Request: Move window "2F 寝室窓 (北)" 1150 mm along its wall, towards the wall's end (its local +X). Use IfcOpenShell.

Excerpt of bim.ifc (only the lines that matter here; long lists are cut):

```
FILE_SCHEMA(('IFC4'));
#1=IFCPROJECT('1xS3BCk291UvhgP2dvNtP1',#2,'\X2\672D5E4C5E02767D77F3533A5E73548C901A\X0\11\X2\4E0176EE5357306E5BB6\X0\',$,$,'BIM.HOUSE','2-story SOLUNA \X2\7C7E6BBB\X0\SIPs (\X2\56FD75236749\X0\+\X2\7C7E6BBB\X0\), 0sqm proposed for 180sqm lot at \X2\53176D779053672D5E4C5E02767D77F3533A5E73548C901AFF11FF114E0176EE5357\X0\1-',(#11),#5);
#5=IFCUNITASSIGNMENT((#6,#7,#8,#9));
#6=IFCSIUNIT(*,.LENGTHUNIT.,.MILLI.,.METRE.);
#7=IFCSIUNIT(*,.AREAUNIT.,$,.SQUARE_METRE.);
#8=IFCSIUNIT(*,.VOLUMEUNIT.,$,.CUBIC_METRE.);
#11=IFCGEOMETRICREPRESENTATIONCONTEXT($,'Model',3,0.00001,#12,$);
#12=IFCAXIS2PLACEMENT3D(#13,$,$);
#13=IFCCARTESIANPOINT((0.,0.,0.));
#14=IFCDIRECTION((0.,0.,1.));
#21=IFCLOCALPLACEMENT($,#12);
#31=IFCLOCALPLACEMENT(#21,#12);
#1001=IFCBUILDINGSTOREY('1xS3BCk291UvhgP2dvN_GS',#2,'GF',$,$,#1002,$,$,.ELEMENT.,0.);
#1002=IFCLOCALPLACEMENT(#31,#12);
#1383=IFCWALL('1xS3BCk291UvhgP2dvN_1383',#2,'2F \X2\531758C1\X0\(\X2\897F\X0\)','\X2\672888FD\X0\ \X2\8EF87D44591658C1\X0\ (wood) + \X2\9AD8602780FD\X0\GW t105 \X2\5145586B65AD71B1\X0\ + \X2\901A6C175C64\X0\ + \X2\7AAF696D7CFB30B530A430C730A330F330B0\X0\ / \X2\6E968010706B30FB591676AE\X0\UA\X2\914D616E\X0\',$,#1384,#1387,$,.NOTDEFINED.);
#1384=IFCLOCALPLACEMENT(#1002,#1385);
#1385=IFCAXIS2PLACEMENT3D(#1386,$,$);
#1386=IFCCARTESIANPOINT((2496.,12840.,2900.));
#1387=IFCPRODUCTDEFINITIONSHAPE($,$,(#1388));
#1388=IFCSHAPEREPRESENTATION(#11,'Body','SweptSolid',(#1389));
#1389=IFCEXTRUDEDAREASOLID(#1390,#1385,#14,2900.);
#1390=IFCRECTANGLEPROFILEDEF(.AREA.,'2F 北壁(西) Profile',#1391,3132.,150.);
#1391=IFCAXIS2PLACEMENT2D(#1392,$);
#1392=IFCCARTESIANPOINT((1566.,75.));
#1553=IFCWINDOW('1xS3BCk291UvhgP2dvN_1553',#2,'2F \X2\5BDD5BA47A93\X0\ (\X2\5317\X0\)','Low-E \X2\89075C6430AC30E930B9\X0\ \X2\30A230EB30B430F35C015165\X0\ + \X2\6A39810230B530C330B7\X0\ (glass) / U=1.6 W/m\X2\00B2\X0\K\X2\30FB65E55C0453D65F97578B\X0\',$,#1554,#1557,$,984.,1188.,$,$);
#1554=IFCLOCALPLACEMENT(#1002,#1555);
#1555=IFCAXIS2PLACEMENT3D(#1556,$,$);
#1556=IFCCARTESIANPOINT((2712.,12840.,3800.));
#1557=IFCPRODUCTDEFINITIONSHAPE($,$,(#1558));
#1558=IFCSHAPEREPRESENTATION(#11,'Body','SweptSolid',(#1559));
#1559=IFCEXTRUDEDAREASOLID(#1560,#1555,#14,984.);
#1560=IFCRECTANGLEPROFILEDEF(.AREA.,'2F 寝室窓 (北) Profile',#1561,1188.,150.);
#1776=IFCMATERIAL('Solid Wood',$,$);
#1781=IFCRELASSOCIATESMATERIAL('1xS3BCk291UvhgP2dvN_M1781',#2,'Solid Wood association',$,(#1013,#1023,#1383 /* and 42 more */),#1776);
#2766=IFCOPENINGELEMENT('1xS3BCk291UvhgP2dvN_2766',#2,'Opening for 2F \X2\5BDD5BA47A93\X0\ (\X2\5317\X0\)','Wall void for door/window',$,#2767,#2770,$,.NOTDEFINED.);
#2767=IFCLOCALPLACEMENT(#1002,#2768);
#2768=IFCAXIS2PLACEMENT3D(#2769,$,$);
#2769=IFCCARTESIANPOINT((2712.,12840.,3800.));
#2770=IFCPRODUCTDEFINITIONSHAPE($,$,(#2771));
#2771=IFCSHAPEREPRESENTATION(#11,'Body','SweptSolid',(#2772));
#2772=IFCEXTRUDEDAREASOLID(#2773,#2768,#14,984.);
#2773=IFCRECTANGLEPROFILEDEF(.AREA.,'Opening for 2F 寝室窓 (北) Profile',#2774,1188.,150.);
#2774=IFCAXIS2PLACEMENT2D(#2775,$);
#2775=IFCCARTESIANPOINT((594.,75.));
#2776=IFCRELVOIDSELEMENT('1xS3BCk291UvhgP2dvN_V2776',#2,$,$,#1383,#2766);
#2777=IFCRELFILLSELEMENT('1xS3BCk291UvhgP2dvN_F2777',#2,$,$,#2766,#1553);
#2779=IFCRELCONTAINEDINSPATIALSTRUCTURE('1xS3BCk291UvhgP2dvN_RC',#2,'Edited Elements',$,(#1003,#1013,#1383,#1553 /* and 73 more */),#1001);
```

```python
import ifcopenshell
import ifcopenshell.api.geometry
import ifcopenshell.util.placement

model = ifcopenshell.open("bim.ifc")

window = model.by_guid("1xS3BCk291UvhgP2dvN_1553")
opening = window.FillsVoids[0].RelatingOpeningElement
wall = opening.VoidsElements[0].RelatingBuildingElement

wall_matrix = ifcopenshell.util.placement.get_local_placement(wall.ObjectPlacement)
shift = wall_matrix[:3, 0] * 1150.0
before = ifcopenshell.util.placement.get_local_placement(window.ObjectPlacement)[:3, 3].copy()

# The window is not placed relative to its opening, so move both.
for product in (opening, window):
    matrix = ifcopenshell.util.placement.get_local_placement(product.ObjectPlacement)
    matrix[:3, 3] += shift
    ifcopenshell.api.geometry.edit_object_placement(model, product=product, matrix=matrix, is_si=False)

after = ifcopenshell.util.placement.get_local_placement(window.ObjectPlacement)[:3, 3]
print("window moved by", (after - before).round(3) + 0.0)

model.write("bim_v2.ifc")
```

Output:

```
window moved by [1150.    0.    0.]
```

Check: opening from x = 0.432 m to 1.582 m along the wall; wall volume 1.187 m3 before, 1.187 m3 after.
